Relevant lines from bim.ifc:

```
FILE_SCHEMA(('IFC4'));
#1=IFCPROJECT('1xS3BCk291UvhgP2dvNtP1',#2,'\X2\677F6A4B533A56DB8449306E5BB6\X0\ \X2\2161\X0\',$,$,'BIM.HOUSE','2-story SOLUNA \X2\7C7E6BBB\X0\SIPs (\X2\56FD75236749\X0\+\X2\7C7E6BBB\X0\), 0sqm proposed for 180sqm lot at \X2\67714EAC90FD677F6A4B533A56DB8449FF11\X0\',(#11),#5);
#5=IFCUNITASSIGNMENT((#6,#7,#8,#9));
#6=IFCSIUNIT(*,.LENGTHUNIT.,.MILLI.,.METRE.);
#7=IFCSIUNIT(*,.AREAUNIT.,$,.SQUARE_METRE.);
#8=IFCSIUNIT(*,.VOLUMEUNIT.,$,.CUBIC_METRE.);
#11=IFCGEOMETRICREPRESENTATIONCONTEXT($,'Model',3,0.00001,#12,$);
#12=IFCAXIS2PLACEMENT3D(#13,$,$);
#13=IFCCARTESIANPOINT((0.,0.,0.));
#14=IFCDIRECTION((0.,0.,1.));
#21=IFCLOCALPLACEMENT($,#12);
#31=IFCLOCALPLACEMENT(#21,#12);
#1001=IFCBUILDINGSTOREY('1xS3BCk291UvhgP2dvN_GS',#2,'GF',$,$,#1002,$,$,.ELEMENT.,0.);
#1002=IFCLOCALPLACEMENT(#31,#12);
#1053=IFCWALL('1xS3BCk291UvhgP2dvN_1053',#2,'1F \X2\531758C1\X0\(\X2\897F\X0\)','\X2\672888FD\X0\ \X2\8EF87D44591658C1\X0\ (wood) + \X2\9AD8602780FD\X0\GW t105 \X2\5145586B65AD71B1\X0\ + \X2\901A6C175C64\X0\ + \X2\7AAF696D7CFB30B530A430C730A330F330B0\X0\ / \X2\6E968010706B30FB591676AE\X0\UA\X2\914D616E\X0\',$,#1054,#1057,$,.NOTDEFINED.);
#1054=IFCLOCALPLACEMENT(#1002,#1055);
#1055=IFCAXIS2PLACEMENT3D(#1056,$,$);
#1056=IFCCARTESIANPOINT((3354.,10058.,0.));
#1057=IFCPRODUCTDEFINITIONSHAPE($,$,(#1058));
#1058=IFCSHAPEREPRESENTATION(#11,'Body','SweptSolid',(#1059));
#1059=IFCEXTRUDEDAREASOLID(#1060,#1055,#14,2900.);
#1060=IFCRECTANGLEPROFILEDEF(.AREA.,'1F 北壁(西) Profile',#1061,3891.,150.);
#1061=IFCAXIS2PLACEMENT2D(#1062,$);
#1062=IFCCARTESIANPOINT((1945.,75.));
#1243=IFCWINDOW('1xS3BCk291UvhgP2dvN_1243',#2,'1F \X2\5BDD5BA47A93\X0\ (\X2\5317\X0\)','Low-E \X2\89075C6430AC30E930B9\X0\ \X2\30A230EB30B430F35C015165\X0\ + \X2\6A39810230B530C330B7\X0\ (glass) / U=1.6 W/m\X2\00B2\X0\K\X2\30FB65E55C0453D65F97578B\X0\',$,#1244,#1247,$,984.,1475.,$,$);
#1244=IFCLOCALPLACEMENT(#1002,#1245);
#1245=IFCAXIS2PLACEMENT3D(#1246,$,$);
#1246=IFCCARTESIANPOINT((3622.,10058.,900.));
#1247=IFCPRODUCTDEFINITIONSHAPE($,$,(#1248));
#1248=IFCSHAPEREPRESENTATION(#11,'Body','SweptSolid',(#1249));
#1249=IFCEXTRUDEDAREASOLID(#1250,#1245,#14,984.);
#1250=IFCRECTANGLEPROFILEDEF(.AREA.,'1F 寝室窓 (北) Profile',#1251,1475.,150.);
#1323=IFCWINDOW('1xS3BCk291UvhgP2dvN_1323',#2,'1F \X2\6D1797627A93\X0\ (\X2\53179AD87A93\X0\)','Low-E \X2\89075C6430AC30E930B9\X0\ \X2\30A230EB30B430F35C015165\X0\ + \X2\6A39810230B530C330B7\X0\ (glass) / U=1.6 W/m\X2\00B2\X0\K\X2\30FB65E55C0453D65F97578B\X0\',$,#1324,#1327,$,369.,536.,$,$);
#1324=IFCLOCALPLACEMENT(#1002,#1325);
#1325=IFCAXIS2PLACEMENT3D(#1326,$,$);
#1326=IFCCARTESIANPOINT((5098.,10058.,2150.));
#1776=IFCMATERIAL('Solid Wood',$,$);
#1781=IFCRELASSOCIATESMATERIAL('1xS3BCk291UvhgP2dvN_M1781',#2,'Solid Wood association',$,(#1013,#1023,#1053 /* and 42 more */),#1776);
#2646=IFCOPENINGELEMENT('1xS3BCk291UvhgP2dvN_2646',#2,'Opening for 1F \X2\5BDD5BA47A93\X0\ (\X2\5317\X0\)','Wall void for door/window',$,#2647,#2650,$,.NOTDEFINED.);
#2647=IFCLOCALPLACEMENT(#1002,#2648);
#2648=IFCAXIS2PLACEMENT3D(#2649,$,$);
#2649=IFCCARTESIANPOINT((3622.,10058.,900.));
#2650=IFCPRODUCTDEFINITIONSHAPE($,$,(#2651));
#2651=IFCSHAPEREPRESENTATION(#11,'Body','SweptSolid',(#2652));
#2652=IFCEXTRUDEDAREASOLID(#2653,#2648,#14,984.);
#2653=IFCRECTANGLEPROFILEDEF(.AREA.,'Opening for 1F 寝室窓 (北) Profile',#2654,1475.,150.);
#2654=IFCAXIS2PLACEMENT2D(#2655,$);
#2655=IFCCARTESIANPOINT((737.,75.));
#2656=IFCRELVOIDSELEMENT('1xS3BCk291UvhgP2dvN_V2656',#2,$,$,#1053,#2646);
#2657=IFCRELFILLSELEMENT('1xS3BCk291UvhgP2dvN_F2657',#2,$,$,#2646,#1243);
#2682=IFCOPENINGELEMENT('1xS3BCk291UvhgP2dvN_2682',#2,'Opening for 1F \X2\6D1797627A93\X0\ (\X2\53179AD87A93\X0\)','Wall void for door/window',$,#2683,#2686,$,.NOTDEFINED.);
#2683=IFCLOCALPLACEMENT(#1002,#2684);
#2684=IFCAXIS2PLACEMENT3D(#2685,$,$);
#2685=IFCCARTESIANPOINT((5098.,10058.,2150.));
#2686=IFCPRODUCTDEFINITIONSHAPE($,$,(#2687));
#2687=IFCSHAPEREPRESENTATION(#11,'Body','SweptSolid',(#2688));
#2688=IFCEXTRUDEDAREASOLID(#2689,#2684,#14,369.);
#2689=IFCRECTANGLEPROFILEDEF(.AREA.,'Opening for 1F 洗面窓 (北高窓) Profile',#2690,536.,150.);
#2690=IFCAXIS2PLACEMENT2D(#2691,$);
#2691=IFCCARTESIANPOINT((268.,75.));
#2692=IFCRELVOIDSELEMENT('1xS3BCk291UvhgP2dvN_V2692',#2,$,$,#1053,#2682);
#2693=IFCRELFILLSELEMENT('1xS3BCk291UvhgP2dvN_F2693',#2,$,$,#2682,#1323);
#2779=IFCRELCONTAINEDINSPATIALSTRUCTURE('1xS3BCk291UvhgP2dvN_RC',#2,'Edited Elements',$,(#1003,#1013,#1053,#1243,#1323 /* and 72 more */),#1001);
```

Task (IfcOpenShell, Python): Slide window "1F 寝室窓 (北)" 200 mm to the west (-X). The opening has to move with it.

```python
import ifcopenshell
import ifcopenshell.api.geometry
import ifcopenshell.util.placement

model = ifcopenshell.open("bim.ifc")

window = model.by_id(1243)
opening = window.FillsVoids[0].RelatingOpeningElement
wall = opening.VoidsElements[0].RelatingBuildingElement

wall_matrix = ifcopenshell.util.placement.get_local_placement(wall.ObjectPlacement)
shift = wall_matrix[:3, 0] * -200.0
before = ifcopenshell.util.placement.get_local_placement(window.ObjectPlacement)[:3, 3].copy()

# The window is not placed relative to its opening, so move both.
for product in (opening, window):
    matrix = ifcopenshell.util.placement.get_local_placement(product.ObjectPlacement)
    matrix[:3, 3] += shift
    ifcopenshell.api.geometry.edit_object_placement(model, product=product, matrix=matrix, is_si=False)

after = ifcopenshell.util.placement.get_local_placement(window.ObjectPlacement)[:3, 3]
print("window moved by", (after - before).round(3) + 0.0)

model.write("bim_rev.ifc")
```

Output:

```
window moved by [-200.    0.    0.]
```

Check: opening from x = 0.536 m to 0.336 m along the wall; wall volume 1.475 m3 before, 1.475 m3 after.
